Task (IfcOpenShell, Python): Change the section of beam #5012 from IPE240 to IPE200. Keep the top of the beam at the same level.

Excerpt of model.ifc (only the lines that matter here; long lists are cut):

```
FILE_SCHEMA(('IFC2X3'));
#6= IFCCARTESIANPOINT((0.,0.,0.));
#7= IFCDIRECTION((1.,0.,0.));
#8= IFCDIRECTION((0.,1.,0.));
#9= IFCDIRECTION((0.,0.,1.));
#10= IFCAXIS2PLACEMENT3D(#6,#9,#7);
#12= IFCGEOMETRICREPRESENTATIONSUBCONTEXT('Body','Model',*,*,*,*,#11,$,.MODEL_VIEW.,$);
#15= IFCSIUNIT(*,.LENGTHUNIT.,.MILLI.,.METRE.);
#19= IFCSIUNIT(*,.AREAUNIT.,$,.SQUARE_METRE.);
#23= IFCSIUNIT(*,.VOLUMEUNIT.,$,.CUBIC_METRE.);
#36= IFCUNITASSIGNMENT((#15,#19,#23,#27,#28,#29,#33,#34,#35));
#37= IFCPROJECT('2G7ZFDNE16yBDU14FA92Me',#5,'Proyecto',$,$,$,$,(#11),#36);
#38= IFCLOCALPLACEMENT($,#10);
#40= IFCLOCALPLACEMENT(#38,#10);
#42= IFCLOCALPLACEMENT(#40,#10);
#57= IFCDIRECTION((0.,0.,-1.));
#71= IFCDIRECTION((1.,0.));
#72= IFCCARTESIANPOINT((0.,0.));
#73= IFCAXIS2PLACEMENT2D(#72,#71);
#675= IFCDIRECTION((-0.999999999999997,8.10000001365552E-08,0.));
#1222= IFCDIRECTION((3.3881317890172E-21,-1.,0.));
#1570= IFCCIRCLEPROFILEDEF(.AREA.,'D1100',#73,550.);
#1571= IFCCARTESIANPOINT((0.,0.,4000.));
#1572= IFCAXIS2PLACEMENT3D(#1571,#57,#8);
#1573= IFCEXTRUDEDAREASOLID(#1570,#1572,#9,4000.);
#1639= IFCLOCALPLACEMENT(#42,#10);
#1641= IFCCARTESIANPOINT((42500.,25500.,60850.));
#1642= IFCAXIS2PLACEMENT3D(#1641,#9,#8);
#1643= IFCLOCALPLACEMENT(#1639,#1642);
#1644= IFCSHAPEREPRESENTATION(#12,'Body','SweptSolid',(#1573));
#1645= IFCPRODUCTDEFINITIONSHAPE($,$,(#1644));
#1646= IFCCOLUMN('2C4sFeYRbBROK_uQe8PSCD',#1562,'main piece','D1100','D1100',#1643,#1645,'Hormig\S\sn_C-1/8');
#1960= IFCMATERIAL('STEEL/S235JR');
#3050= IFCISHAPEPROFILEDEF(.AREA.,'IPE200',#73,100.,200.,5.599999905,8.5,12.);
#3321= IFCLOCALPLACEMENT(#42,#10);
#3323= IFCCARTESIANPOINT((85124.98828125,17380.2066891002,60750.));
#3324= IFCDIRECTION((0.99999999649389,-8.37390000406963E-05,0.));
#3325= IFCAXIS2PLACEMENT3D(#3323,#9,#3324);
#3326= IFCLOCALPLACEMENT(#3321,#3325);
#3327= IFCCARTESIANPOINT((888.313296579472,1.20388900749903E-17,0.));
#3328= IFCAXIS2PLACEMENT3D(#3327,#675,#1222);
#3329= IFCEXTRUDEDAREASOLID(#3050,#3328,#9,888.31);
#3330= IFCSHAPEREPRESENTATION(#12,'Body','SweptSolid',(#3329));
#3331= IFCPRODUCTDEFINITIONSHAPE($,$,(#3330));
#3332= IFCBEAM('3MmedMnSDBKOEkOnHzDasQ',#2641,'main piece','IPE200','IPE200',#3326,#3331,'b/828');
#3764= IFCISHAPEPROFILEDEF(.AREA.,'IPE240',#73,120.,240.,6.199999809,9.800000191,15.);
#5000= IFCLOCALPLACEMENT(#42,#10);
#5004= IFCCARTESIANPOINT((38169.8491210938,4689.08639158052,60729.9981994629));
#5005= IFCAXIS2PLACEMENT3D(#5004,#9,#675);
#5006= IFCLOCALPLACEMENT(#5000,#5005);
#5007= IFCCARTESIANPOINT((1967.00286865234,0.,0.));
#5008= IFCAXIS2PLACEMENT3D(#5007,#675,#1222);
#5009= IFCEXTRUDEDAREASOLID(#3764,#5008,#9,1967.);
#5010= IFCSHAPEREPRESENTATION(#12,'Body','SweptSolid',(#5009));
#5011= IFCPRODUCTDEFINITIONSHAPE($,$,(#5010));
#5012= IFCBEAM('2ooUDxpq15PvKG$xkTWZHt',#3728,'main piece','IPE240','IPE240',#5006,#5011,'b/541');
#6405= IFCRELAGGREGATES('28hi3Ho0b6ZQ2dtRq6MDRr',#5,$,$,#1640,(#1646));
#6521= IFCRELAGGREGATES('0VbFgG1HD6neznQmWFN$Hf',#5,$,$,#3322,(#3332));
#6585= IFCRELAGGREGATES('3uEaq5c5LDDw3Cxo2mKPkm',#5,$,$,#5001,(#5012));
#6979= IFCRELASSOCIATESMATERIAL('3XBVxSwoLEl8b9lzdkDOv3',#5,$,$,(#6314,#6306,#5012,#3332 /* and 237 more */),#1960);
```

```python
import ifcopenshell
import ifcopenshell.util.element
import ifcopenshell.util.representation

model = ifcopenshell.open("model.ifc")

member = model.by_id(5012)
source = next(p for p in model.by_type("IfcIShapeProfileDef") if p.ProfileName == "IPE200")

body = ifcopenshell.util.representation.get_representation(member, "Model", "Body")
solid = body.Items[0]
old_profile = solid.SweptArea

# Copy the section's sizes but keep this member's own profile position.
profile = ifcopenshell.util.element.copy(model, source)
# Profiles are centred, so shift by half the change in depth to hold the top.
shift = (old_profile.OverallDepth - profile.OverallDepth) / 2
x, y = old_profile.Position.Location.Coordinates
up = (0.0, 1.0)  # upwards, in the solid's own plane
location = model.createIfcCartesianPoint((x + up[0] * shift, y + up[1] * shift))
profile.Position = model.createIfcAxis2Placement2D(location, old_profile.Position.RefDirection)
solid.SweptArea = profile
if not model.get_total_inverses(old_profile):
    ifcopenshell.util.element.remove_deep2(model, old_profile)
member.Description = member.Description.replace("IPE240", "IPE200")
member.ObjectType = member.ObjectType.replace("IPE240", "IPE200")

print(solid.SweptArea)

model.write("model_v2.ifc")
```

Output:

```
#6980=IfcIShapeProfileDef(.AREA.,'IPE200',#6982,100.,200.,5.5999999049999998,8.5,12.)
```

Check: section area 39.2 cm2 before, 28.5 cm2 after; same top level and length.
